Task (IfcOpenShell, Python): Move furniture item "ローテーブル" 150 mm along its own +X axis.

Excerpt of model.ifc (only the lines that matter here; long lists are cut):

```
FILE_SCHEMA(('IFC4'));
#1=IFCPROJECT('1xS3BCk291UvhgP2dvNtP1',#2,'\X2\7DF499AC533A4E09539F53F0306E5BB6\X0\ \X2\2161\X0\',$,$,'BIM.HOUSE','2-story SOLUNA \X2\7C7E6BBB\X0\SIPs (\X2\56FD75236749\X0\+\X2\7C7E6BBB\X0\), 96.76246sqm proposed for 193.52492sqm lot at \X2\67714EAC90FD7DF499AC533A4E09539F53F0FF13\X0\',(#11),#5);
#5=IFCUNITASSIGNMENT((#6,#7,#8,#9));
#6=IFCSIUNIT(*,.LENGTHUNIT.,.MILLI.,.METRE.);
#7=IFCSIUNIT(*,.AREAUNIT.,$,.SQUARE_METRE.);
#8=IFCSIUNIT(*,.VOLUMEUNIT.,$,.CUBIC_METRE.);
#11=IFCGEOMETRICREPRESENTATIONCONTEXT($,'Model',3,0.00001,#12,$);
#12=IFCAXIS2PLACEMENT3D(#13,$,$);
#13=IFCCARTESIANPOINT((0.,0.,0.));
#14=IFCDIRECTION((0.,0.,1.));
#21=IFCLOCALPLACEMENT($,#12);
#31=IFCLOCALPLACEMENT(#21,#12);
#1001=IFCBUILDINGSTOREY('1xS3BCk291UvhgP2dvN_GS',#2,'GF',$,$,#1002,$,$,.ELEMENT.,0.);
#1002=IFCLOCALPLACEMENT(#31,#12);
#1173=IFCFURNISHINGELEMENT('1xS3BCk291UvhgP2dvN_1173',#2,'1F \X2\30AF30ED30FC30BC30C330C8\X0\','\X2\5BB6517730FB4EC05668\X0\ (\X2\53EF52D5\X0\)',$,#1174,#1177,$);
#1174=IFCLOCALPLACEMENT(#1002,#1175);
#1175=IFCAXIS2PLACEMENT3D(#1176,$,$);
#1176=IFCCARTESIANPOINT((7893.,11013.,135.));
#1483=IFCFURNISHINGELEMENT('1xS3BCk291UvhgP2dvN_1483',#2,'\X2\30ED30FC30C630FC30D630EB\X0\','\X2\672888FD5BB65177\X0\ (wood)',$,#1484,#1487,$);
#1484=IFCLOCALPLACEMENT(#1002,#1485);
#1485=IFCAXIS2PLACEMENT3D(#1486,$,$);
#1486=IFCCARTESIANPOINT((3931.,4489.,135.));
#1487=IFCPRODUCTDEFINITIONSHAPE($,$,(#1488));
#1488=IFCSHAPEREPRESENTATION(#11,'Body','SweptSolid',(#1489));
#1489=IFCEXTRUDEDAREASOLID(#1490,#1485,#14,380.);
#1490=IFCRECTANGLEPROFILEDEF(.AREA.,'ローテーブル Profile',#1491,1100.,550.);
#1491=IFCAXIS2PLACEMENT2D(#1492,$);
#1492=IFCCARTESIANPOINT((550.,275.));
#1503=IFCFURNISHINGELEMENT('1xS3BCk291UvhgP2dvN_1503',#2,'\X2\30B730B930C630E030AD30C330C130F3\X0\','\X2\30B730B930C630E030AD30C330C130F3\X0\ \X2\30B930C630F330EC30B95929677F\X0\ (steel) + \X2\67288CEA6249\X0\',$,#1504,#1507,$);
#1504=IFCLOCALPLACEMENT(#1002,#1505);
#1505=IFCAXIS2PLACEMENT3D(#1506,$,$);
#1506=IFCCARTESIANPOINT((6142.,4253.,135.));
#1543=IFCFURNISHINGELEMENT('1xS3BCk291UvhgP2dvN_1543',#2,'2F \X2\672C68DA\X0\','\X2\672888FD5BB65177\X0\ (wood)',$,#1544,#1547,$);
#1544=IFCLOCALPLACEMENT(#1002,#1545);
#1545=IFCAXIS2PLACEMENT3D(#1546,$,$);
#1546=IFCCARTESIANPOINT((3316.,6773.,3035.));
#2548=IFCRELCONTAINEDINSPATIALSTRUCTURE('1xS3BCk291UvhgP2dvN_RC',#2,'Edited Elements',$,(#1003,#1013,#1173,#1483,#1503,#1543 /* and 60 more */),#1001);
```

```python
import ifcopenshell
import ifcopenshell.api.geometry
import ifcopenshell.util.placement

model = ifcopenshell.open("model.ifc")

item = model.by_guid("1xS3BCk291UvhgP2dvN_1483")
matrix = ifcopenshell.util.placement.get_local_placement(item.ObjectPlacement)
matrix[:3, 3] += matrix[:3, 0] * 150.0
ifcopenshell.api.geometry.edit_object_placement(model, product=item, matrix=matrix, is_si=False)

print(ifcopenshell.util.placement.get_local_placement(item.ObjectPlacement).round(3) + 0.0)

model.write("model_v2.ifc")
```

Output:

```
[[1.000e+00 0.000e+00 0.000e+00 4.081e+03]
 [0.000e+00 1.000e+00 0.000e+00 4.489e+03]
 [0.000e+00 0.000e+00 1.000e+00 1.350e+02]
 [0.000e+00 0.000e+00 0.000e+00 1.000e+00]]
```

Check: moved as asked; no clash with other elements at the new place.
